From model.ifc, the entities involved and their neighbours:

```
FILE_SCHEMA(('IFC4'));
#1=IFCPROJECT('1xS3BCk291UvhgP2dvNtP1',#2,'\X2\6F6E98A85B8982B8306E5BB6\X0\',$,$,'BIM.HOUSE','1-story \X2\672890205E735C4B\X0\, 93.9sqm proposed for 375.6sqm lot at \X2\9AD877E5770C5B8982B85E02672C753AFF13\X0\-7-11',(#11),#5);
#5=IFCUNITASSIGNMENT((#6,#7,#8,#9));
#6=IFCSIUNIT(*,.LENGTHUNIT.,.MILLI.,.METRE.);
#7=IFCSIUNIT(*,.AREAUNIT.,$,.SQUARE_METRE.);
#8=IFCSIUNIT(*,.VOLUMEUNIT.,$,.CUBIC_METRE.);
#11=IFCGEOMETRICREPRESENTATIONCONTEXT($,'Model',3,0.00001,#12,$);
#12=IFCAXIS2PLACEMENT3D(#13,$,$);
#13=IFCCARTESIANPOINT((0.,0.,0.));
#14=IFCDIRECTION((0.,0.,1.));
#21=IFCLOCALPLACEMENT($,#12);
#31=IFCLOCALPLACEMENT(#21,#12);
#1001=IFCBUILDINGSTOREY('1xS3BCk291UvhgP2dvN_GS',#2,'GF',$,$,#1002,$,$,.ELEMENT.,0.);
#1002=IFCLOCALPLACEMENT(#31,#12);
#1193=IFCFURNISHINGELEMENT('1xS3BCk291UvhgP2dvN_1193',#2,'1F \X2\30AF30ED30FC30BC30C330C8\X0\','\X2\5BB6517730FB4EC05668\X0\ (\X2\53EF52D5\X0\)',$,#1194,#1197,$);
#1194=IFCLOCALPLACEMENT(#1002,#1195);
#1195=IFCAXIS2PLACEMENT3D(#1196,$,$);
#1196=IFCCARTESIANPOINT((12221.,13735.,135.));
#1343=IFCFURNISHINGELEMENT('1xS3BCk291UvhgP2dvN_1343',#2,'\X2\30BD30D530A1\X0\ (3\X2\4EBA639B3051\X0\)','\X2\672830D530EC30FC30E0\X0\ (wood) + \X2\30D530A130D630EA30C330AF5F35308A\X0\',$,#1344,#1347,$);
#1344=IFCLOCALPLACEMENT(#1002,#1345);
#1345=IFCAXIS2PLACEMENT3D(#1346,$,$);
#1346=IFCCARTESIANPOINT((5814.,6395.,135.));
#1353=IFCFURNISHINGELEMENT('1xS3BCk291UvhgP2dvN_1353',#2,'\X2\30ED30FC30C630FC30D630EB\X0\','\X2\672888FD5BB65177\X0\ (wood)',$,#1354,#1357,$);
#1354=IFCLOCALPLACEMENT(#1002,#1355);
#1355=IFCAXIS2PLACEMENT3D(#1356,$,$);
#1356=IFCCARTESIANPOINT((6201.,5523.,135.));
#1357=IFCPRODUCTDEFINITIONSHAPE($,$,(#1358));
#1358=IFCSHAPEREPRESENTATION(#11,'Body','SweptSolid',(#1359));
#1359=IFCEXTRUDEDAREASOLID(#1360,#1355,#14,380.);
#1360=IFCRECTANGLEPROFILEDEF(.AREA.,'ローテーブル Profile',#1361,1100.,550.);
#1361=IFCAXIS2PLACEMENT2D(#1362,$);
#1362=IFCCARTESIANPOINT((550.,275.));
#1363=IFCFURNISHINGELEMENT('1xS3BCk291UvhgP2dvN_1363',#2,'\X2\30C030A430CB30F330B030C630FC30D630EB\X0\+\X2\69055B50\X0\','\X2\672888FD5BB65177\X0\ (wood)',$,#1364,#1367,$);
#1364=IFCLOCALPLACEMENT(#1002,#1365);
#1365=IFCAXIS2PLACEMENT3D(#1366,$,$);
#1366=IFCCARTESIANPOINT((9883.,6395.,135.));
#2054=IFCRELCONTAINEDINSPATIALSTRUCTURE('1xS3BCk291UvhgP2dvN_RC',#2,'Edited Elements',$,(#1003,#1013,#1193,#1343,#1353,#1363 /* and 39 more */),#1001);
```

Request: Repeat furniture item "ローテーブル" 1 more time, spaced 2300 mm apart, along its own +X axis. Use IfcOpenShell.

```python
import ifcopenshell
import ifcopenshell.api.geometry
import ifcopenshell.api.root
import ifcopenshell.util.element
import ifcopenshell.util.placement
import ifcopenshell.util.unit

model = ifcopenshell.open("model.ifc")
unit_scale = ifcopenshell.util.unit.calculate_unit_scale(model)


def reuse_history(source, copy):
    """copy_class also copies each property set's owner history, people and application; keep the originals."""
    for rel in copy.IsDefinedBy:
        if rel.is_a("IfcRelDefinesByProperties") and (history := rel.RelatingPropertyDefinition.OwnerHistory):
            rel.RelatingPropertyDefinition.OwnerHistory = source.OwnerHistory
            ifcopenshell.util.element.remove_deep2(model, history)


source = model.by_id(1353)
base = ifcopenshell.util.placement.get_local_placement(source.ObjectPlacement)
step = base[:3, 0] * 2.3 / unit_scale

for i in range(1, 2):
    copy = ifcopenshell.api.root.copy_class(model, product=source)
    copy.Representation = ifcopenshell.util.element.copy_deep(
        model, source.Representation, exclude=["IfcGeometricRepresentationContext", "IfcRepresentationMap"]
    )
    reuse_history(source, copy)
    matrix = base.copy()
    matrix[:3, 3] += i * step
    print("added at", matrix[:3, 3].round(3) + 0.0)
    ifcopenshell.api.geometry.edit_object_placement(model, product=copy, matrix=matrix, is_si=False)

model.write("model_edited.ifc")
```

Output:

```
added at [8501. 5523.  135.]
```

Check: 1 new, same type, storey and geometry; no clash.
